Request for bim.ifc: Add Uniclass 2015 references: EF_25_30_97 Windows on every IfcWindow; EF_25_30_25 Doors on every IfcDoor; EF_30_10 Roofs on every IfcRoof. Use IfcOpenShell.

First a look at what the model holds.

```python
import ifcopenshell

model = ifcopenshell.open("bim.ifc")
print(model.schema)
print("classifications:", [c.Name for c in model.by_type("IfcClassification")])
for ifc_class in ("IfcDoor", "IfcRoof", "IfcStair", "IfcWall", "IfcWindow"):
    print(ifc_class, len(model.by_type(ifc_class)))
```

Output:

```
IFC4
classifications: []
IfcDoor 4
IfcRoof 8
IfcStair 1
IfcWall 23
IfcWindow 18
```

```python
import ifcopenshell
import ifcopenshell.api.classification

model = ifcopenshell.open("bim.ifc")

system = ifcopenshell.api.classification.add_classification(model, classification="Uniclass 2015")

codes = {
    "IfcWindow": ("EF_25_30_97", "Windows"),
    "IfcDoor": ("EF_25_30_25", "Doors"),
    "IfcRoof": ("EF_30_10", "Roofs"),
}
for ifc_class, (code, name) in codes.items():
    products = model.by_type(ifc_class)
    ifcopenshell.api.classification.add_reference(
        model, products=products, classification=system, identification=code, name=name
    )
    print(code, len(products))

model.write("bim_edited.ifc")
```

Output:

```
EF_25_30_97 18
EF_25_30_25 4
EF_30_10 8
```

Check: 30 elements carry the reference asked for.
